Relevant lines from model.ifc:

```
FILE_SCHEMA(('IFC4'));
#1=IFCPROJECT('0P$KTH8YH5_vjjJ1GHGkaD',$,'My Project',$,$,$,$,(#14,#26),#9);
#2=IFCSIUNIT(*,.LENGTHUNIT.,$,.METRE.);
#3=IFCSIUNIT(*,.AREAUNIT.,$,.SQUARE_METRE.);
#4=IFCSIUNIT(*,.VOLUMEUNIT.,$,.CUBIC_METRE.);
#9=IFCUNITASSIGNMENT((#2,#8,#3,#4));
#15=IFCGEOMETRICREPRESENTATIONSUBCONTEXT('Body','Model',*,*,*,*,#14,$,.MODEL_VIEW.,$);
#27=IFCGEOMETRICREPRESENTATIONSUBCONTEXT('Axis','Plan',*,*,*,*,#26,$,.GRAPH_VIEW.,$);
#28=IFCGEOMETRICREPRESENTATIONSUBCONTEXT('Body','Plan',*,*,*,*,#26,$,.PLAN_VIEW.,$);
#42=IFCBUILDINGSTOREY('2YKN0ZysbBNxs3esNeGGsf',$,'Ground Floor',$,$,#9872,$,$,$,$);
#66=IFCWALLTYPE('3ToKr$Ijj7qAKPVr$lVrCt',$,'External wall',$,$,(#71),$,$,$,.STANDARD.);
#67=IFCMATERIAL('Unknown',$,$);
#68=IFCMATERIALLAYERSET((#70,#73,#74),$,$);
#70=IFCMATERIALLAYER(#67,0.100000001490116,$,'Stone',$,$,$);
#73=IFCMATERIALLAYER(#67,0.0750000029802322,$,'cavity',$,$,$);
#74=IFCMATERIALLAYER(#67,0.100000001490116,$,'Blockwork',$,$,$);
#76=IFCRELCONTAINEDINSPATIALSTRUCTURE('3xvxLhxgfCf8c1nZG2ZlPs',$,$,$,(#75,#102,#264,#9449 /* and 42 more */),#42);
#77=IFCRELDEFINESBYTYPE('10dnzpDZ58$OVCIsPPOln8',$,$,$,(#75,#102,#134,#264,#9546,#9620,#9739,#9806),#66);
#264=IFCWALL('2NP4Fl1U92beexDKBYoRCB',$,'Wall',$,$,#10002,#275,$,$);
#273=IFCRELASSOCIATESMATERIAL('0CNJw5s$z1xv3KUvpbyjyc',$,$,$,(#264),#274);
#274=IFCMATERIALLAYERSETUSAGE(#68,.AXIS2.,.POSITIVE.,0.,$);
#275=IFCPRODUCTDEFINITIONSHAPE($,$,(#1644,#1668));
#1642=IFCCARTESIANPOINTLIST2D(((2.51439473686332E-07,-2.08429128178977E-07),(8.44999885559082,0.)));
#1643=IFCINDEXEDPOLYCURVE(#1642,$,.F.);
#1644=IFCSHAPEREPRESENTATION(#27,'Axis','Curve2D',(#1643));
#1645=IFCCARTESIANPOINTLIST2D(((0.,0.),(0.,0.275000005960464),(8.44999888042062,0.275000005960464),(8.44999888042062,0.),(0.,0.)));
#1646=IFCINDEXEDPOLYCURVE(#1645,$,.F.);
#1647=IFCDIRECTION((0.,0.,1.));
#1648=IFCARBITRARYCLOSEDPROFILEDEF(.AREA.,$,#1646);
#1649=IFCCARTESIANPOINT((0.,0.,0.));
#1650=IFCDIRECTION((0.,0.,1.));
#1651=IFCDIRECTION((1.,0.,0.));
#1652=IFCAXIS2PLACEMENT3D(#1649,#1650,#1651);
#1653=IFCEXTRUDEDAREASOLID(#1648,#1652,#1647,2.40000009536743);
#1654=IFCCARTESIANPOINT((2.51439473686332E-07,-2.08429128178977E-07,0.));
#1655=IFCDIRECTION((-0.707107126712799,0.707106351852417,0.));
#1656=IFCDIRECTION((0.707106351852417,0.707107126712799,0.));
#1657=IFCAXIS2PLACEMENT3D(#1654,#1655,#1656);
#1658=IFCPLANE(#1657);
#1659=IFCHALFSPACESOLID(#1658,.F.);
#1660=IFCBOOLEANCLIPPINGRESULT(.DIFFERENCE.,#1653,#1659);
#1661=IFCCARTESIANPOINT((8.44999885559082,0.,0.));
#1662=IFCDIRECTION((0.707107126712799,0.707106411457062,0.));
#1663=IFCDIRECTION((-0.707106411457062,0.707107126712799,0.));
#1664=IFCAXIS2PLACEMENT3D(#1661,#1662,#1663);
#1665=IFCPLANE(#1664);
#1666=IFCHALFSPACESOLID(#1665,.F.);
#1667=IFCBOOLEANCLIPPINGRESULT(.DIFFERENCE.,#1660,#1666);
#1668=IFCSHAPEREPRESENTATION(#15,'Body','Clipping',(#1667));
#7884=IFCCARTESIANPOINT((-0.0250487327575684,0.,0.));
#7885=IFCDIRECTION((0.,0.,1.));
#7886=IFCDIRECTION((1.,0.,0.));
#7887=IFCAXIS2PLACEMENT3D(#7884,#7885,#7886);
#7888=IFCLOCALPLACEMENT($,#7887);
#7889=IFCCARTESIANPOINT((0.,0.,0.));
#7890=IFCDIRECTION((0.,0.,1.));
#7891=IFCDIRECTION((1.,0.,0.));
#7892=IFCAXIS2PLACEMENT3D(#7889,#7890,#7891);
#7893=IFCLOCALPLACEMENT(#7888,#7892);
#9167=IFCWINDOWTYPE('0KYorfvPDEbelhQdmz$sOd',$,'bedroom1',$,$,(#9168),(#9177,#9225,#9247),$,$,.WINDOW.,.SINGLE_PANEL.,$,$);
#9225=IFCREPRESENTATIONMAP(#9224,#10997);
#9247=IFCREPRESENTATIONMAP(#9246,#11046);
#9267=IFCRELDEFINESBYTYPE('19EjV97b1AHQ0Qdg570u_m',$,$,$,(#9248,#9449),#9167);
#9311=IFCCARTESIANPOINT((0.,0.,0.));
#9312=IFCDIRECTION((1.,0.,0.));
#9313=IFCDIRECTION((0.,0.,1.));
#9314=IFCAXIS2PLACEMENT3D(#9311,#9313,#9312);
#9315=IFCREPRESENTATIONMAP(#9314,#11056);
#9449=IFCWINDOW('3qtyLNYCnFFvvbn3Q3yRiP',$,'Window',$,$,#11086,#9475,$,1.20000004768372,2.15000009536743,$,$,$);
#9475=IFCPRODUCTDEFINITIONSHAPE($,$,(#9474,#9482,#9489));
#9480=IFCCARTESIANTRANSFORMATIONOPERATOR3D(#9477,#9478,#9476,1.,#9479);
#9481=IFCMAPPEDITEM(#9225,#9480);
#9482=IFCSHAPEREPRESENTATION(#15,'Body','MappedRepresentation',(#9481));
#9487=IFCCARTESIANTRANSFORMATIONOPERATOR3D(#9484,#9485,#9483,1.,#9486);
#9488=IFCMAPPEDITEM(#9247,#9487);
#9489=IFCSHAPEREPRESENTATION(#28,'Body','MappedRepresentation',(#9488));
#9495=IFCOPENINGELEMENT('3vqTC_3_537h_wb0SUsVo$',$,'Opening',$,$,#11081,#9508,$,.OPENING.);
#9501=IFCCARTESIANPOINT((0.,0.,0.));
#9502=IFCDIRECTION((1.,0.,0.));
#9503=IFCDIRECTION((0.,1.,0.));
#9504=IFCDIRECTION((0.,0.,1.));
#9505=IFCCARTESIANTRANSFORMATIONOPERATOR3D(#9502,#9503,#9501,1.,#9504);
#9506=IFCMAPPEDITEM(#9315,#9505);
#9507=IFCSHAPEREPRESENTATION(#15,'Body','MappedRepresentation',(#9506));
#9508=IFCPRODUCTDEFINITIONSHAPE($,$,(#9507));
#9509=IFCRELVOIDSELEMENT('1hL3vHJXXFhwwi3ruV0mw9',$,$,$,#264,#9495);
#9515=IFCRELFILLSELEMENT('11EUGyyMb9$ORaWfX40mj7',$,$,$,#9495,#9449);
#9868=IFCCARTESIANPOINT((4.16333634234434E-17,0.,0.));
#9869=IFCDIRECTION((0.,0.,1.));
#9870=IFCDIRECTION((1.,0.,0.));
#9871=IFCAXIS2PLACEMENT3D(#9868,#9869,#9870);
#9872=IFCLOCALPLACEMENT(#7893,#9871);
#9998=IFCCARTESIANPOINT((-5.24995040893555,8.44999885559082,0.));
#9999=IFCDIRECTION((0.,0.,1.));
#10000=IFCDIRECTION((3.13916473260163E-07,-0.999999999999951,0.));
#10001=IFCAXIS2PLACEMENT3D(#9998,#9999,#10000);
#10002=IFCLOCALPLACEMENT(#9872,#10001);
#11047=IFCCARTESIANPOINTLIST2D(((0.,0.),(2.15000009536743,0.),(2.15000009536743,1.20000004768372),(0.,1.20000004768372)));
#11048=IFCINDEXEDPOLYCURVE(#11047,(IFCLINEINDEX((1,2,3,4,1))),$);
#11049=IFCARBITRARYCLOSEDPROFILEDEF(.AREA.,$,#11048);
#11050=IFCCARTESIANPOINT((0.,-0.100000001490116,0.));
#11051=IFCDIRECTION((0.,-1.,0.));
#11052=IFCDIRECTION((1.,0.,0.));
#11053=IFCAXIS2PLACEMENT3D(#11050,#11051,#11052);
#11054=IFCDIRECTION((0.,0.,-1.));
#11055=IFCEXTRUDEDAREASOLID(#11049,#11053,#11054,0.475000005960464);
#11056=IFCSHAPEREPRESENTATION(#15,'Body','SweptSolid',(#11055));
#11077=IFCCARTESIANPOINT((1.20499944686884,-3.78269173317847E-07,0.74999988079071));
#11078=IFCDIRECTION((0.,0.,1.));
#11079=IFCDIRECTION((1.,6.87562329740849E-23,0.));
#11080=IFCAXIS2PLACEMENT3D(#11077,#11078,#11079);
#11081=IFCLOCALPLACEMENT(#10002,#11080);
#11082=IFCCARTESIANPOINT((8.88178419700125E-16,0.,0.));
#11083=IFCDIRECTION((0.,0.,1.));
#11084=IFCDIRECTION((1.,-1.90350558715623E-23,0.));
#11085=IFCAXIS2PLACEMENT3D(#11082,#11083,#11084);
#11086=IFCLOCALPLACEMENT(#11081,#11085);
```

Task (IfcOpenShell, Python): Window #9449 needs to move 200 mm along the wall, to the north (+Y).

```python
import ifcopenshell
import ifcopenshell.api.geometry
import ifcopenshell.util.placement
import ifcopenshell.util.unit

model = ifcopenshell.open("model.ifc")
unit_scale = ifcopenshell.util.unit.calculate_unit_scale(model)

window = model.by_id(9449)
opening = window.FillsVoids[0].RelatingOpeningElement
wall = opening.VoidsElements[0].RelatingBuildingElement

wall_matrix = ifcopenshell.util.placement.get_local_placement(wall.ObjectPlacement)
shift = wall_matrix[:3, 0] * -0.2 / unit_scale
before = ifcopenshell.util.placement.get_local_placement(window.ObjectPlacement)[:3, 3].copy()

# The window is placed relative to its opening, so it follows when the opening moves.
matrix = ifcopenshell.util.placement.get_local_placement(opening.ObjectPlacement)
matrix[:3, 3] += shift
ifcopenshell.api.geometry.edit_object_placement(
    model, product=opening, matrix=matrix, is_si=False, should_transform_children=True
)

after = ifcopenshell.util.placement.get_local_placement(window.ObjectPlacement)[:3, 3]
print("window moved by", (after - before).round(3) + 0.0)

model.write("model_edited.ifc")
```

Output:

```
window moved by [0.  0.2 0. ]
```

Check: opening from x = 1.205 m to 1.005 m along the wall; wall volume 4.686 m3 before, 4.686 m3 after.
